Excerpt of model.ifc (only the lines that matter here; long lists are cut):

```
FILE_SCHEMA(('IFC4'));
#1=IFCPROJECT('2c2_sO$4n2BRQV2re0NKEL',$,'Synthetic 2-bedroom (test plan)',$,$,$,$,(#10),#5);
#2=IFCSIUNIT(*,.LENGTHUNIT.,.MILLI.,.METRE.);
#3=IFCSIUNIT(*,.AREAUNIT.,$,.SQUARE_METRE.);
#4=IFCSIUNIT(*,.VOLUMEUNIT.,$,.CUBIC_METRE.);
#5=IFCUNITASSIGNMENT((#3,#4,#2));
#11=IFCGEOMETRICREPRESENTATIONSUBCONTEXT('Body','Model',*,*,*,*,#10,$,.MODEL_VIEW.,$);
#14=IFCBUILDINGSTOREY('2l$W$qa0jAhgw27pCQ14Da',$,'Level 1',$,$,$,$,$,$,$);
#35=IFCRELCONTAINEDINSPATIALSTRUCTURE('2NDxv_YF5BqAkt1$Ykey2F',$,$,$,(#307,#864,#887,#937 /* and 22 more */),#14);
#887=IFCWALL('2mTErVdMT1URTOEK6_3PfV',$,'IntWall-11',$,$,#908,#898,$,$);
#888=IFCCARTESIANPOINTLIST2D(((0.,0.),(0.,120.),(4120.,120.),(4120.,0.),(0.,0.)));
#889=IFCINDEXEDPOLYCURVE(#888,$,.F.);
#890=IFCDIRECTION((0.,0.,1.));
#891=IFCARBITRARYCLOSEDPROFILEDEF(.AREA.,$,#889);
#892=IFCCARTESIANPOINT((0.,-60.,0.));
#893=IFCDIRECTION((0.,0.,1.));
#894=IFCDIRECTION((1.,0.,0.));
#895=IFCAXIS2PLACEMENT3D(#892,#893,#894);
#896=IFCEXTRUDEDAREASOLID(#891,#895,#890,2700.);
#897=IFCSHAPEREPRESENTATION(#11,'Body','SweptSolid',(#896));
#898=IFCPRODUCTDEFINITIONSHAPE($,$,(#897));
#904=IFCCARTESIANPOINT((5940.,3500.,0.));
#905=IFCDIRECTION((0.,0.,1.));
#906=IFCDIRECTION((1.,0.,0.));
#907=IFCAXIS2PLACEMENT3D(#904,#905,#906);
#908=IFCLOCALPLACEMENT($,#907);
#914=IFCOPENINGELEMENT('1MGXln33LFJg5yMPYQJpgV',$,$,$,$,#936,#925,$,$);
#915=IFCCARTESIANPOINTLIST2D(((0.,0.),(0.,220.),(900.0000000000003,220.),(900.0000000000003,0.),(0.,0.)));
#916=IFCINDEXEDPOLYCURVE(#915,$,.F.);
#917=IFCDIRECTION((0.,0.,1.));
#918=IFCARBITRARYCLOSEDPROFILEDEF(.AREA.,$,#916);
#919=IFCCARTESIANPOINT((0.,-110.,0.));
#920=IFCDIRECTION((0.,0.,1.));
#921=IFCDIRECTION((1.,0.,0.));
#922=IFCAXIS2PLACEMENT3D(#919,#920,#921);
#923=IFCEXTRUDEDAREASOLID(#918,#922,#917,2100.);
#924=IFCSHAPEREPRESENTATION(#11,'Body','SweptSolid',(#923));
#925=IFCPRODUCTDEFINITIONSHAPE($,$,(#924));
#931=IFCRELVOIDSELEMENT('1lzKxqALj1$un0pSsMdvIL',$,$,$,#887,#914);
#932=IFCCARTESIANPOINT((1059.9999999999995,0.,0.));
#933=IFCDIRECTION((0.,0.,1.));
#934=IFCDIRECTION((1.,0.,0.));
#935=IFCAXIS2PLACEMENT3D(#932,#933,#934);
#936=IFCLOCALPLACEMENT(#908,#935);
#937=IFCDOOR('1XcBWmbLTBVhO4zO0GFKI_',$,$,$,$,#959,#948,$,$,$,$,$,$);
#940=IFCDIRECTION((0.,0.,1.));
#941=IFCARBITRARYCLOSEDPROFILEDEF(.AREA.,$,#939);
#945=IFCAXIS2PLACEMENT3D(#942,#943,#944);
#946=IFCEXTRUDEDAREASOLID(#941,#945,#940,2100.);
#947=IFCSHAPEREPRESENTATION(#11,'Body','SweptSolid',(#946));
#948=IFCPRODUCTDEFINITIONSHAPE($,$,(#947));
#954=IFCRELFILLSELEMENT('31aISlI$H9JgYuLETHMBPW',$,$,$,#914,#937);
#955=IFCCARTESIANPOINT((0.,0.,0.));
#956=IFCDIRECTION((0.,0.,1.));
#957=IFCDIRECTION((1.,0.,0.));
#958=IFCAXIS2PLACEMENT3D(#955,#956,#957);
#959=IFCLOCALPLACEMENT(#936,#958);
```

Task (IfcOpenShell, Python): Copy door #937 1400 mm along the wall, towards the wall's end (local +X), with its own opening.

```python
import ifcopenshell
import ifcopenshell.api.feature
import ifcopenshell.api.geometry
import ifcopenshell.api.root
import ifcopenshell.geom
import ifcopenshell.util.element
import ifcopenshell.util.placement
import ifcopenshell.util.shape
import ifcopenshell.util.unit

model = ifcopenshell.open("model.ifc")
unit_scale = ifcopenshell.util.unit.calculate_unit_scale(model)
settings = ifcopenshell.geom.settings()


def volume(element):
    """Net volume in cubic metres, openings subtracted."""
    shape = ifcopenshell.geom.create_shape(settings, element)
    return ifcopenshell.util.shape.get_volume(shape.geometry)


door = model.by_guid("1XcBWmbLTBVhO4zO0GFKI_")
opening = door.FillsVoids[0].RelatingOpeningElement
wall = opening.VoidsElements[0].RelatingBuildingElement
before = volume(wall)
shift = ifcopenshell.util.placement.get_local_placement(wall.ObjectPlacement)[:3, 0] * 1.4 / unit_scale

# copy_class copies the void relationship, type, container and properties, but no geometry.
new_opening = ifcopenshell.api.root.copy_class(model, product=opening)
new_opening.Representation = ifcopenshell.util.element.copy_deep(
    model, opening.Representation, exclude=["IfcGeometricRepresentationContext", "IfcRepresentationMap"]
)
new_door = ifcopenshell.api.root.copy_class(model, product=door)
new_door.Representation = ifcopenshell.util.element.copy_deep(
    model, door.Representation, exclude=["IfcGeometricRepresentationContext", "IfcRepresentationMap"]
)
ifcopenshell.api.feature.add_filling(model, opening=new_opening, element=new_door)

for old, new in ((opening, new_opening), (door, new_door)):
    matrix = ifcopenshell.util.placement.get_local_placement(old.ObjectPlacement)
    matrix[:3, 3] += shift
    ifcopenshell.api.geometry.edit_object_placement(model, product=new, matrix=matrix, is_si=False)

after = volume(wall)

print(f"wall volume {before:.3f} -> {after:.3f} m3")

model.write("model-out.ifc")
```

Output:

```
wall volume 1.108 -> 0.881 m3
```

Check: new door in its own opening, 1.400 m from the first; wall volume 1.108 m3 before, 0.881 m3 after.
